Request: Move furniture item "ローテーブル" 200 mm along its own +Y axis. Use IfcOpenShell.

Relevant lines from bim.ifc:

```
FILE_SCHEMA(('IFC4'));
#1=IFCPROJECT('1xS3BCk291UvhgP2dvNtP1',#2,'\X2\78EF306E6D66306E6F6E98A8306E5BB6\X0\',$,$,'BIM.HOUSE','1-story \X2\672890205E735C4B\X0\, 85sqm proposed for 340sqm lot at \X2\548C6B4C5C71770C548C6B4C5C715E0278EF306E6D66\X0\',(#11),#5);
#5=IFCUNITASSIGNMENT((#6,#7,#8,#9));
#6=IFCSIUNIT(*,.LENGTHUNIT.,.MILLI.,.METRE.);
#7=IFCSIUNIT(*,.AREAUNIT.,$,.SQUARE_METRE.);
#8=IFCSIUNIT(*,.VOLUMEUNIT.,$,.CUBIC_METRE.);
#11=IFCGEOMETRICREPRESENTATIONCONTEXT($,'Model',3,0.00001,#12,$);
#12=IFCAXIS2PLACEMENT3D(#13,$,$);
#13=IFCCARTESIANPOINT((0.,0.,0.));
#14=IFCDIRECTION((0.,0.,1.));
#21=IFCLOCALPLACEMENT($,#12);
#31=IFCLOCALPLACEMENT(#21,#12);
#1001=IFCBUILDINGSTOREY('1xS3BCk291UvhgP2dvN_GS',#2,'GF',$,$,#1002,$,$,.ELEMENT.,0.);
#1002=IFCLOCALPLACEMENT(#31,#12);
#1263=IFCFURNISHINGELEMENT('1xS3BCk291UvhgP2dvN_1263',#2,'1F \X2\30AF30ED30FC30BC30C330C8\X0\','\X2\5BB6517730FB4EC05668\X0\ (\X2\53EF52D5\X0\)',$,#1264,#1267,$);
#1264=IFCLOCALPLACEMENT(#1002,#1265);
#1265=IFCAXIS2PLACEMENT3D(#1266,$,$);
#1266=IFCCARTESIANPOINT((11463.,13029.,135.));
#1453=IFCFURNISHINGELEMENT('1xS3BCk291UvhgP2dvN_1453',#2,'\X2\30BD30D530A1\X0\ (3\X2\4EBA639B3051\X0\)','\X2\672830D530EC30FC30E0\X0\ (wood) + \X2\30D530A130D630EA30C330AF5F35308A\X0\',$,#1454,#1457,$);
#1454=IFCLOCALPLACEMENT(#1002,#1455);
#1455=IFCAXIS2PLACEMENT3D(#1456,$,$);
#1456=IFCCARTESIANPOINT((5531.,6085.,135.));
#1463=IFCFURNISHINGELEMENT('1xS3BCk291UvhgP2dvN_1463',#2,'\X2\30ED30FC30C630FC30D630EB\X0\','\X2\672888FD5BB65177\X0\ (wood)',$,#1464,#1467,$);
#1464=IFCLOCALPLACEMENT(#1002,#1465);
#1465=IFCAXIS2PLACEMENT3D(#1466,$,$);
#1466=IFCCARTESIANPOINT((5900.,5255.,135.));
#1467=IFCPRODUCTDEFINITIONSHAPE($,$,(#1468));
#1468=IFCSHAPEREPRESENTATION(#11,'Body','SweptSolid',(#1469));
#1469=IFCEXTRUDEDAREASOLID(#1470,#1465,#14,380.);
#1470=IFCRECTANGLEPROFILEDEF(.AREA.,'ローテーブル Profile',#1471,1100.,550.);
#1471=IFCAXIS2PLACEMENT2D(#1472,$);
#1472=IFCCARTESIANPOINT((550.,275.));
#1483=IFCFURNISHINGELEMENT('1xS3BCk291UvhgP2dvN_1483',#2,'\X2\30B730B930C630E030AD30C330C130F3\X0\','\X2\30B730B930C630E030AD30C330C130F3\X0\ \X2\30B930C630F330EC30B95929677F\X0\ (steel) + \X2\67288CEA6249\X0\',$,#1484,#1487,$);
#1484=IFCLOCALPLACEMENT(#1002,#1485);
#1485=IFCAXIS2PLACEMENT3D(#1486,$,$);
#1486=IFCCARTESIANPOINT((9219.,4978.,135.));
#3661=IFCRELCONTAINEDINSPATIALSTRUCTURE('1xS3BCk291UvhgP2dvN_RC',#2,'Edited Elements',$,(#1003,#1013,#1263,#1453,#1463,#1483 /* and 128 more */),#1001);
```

```python
import ifcopenshell
import ifcopenshell.api.geometry
import ifcopenshell.util.placement
import ifcopenshell.util.unit

model = ifcopenshell.open("bim.ifc")
unit_scale = ifcopenshell.util.unit.calculate_unit_scale(model)

item = model.by_id(1463)
matrix = ifcopenshell.util.placement.get_local_placement(item.ObjectPlacement)
matrix[:3, 3] += matrix[:3, 1] * 0.2 / unit_scale
ifcopenshell.api.geometry.edit_object_placement(model, product=item, matrix=matrix, is_si=False)

print(ifcopenshell.util.placement.get_local_placement(item.ObjectPlacement).round(3) + 0.0)

model.write("bim-out.ifc")
```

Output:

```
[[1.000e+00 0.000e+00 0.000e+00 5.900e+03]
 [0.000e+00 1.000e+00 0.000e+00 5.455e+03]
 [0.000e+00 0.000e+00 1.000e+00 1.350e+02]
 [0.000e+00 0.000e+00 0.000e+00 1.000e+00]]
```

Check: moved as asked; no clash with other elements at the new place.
